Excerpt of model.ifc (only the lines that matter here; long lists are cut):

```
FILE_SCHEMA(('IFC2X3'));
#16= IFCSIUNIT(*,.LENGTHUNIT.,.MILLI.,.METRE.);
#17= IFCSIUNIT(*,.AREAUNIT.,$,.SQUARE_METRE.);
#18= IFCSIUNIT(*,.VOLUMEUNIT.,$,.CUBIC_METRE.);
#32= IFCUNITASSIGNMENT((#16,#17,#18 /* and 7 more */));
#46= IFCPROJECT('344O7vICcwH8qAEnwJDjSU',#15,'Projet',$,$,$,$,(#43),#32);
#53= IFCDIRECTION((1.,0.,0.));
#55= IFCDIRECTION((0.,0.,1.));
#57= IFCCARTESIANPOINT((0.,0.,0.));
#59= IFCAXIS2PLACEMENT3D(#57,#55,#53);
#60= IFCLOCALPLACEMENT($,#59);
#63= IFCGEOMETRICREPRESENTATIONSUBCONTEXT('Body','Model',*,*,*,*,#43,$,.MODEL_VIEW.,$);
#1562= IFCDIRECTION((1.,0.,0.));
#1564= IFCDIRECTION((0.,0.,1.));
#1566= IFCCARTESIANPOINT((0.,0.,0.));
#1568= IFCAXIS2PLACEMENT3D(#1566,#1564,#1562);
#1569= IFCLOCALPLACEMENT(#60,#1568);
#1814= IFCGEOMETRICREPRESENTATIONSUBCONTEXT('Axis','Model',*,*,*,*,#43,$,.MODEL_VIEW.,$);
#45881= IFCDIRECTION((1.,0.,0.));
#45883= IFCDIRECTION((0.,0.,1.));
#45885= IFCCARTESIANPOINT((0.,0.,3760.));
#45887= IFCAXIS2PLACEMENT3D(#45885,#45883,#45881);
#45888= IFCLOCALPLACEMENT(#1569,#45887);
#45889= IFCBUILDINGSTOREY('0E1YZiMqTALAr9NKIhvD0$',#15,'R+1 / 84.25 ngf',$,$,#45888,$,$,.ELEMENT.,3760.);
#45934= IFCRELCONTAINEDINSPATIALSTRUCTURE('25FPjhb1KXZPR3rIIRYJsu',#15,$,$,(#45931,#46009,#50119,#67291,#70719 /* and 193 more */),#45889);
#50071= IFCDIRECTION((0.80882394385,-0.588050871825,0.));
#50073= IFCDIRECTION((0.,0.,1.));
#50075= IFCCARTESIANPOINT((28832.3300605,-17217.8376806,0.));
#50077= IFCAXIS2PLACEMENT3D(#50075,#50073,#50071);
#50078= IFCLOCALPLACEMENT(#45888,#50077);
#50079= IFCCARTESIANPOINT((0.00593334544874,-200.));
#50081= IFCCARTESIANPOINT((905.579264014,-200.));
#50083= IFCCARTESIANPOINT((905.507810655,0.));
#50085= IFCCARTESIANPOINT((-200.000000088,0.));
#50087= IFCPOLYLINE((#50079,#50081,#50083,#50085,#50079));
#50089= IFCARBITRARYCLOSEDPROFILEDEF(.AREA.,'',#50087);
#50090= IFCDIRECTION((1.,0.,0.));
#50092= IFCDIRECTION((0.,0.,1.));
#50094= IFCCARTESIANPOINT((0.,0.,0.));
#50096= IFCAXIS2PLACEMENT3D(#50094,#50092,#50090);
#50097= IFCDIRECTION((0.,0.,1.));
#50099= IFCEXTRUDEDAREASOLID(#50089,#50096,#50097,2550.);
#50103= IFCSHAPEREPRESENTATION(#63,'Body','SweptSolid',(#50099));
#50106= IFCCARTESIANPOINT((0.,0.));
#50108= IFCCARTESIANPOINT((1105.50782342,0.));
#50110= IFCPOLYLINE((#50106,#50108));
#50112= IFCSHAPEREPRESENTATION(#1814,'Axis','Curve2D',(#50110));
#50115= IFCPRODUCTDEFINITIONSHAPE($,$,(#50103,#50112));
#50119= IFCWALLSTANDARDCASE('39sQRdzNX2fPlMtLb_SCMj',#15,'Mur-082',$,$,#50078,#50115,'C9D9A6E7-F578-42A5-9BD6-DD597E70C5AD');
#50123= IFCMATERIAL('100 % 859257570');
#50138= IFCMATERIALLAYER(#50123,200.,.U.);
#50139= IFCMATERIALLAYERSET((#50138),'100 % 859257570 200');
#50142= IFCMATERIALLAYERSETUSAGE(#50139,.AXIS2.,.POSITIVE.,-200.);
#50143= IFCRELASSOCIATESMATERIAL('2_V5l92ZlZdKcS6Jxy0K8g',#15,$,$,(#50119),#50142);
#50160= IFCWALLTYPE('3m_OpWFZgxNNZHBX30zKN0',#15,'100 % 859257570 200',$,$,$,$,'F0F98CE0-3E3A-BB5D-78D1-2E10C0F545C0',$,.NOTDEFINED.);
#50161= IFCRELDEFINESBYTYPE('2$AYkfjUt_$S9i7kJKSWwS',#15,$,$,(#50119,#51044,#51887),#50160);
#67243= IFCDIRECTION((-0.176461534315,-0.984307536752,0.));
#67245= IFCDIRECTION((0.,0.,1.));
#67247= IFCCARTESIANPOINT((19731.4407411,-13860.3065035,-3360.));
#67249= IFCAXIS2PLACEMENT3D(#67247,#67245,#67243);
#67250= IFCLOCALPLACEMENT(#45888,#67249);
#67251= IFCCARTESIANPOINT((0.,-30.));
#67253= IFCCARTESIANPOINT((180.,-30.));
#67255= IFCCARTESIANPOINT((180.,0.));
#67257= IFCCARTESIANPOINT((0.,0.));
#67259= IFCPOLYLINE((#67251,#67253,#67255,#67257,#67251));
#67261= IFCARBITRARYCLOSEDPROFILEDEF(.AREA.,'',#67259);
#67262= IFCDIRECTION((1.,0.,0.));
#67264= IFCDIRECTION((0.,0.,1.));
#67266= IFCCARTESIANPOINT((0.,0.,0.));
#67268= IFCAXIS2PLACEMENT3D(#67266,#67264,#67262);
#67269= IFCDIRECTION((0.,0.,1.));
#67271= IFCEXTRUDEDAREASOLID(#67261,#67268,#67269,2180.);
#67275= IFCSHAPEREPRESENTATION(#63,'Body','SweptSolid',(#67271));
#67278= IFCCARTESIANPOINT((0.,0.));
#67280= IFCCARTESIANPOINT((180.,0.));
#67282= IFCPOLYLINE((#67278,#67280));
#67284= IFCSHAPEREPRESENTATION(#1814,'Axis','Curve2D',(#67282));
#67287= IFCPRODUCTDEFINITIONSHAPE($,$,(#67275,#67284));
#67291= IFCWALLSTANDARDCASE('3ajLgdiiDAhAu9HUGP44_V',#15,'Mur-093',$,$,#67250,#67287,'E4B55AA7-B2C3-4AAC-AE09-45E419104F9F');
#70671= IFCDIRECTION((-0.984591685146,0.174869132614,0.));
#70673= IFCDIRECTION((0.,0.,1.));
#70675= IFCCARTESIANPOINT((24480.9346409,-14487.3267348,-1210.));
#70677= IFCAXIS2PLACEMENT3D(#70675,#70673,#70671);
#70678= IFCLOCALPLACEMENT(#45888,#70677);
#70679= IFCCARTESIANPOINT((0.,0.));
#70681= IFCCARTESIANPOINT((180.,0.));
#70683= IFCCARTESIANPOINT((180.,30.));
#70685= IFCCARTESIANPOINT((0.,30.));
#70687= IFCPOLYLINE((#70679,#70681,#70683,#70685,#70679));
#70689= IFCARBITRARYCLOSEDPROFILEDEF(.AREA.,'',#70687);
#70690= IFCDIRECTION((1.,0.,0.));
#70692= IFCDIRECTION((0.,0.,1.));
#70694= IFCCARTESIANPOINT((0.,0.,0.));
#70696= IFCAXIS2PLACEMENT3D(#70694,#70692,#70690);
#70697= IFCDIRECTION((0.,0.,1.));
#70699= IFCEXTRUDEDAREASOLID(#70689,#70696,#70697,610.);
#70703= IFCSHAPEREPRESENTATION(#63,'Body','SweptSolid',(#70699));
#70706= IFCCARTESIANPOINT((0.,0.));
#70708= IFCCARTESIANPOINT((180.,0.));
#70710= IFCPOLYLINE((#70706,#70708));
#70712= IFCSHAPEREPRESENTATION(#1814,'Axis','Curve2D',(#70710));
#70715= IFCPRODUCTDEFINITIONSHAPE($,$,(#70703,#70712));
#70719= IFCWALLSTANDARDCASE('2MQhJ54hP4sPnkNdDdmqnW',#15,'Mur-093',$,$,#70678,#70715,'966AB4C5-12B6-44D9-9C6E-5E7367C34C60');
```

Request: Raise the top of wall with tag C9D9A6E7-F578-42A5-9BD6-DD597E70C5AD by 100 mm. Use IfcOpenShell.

```python
import ifcopenshell
import ifcopenshell.geom
import ifcopenshell.util.representation
import ifcopenshell.util.shape
import ifcopenshell.util.unit

model = ifcopenshell.open("model.ifc")
unit_scale = ifcopenshell.util.unit.calculate_unit_scale(model)
settings = ifcopenshell.geom.settings()


def volume(element):
    """Net volume in cubic metres, openings subtracted."""
    shape = ifcopenshell.geom.create_shape(settings, element)
    return ifcopenshell.util.shape.get_volume(shape.geometry)


wall = model.by_id(50119)
before = volume(wall)

body = ifcopenshell.util.representation.get_representation(wall, "Model", "Body")
solid = body.Items[0]
old_height = solid.Depth
solid.Depth += 0.1 / unit_scale
after = volume(wall)

print(f"height {old_height:g} -> {solid.Depth:g}, volume {before:.3f} -> {after:.3f} m3")

model.write("model-out.ifc")
```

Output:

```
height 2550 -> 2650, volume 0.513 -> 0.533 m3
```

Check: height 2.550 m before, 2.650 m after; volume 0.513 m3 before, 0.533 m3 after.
